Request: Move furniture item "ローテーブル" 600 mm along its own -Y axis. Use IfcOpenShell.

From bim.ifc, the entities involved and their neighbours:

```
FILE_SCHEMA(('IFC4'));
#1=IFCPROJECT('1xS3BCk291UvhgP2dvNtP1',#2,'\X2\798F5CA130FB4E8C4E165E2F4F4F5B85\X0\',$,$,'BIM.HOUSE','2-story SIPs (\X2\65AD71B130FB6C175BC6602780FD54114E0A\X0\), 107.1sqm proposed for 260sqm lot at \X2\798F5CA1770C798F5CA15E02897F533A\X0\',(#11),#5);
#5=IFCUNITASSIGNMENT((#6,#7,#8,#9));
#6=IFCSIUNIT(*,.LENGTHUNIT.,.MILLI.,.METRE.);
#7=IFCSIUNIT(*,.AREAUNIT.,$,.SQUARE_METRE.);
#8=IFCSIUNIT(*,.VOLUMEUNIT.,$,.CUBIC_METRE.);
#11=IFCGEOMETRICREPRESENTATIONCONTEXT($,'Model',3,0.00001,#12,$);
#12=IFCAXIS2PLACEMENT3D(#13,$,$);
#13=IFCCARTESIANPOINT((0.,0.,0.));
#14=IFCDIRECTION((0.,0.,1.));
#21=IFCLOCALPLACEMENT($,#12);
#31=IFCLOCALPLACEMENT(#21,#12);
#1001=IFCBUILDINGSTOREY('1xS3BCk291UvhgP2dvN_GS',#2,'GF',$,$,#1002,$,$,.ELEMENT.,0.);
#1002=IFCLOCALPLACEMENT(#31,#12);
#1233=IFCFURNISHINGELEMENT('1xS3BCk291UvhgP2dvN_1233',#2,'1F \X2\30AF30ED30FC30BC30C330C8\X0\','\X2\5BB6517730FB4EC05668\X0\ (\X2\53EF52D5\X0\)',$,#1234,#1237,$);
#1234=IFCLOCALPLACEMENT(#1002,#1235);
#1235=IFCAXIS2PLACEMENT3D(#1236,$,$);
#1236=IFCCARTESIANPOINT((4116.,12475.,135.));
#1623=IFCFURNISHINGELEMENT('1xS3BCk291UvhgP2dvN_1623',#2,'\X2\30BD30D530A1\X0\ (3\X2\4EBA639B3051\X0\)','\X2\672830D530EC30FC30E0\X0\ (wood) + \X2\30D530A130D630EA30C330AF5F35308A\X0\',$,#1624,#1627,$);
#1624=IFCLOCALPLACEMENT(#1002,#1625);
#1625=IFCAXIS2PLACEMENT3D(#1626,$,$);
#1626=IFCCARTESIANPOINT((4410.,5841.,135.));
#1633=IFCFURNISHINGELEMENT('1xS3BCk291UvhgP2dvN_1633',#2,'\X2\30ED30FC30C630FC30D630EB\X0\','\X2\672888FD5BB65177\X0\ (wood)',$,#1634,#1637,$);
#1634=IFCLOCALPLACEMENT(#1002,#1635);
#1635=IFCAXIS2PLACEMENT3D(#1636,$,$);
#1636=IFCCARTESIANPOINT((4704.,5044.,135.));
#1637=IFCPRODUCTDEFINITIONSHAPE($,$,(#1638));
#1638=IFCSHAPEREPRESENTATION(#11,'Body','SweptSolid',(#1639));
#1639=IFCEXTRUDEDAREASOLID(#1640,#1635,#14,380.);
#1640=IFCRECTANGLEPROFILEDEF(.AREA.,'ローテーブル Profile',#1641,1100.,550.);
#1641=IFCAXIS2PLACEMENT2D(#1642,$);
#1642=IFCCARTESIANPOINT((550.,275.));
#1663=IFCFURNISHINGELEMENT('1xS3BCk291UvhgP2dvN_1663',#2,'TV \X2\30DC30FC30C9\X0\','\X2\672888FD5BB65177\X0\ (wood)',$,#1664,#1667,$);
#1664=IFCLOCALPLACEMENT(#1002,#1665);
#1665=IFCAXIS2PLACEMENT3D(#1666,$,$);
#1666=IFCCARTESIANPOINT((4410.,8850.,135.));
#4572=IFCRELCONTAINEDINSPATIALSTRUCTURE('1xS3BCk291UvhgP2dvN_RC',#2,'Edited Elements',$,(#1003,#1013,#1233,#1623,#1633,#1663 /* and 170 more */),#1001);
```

```python
import ifcopenshell
import ifcopenshell.api.geometry
import ifcopenshell.util.placement
import ifcopenshell.util.unit

model = ifcopenshell.open("bim.ifc")
unit_scale = ifcopenshell.util.unit.calculate_unit_scale(model)

item = model.by_guid("1xS3BCk291UvhgP2dvN_1633")
matrix = ifcopenshell.util.placement.get_local_placement(item.ObjectPlacement)
matrix[:3, 3] -= matrix[:3, 1] * 0.6 / unit_scale
ifcopenshell.api.geometry.edit_object_placement(model, product=item, matrix=matrix, is_si=False)

print(ifcopenshell.util.placement.get_local_placement(item.ObjectPlacement).round(3) + 0.0)

model.write("bim_updated.ifc")
```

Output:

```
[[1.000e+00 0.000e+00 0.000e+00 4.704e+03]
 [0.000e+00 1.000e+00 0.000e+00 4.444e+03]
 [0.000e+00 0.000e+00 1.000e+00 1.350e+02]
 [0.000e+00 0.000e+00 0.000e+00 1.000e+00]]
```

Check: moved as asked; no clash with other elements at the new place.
